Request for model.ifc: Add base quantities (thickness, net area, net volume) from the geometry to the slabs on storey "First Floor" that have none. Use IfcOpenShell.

First a look at what the model holds.

```python
import ifcopenshell
import ifcopenshell.util.element
import ifcopenshell.util.unit

model = ifcopenshell.open("model.ifc")
print(model.schema)
for unit_type in ("LENGTHUNIT", "AREAUNIT", "VOLUMEUNIT"):
    print(unit_type, ifcopenshell.util.unit.calculate_unit_scale(model, unit_type))
storey = next(s for s in model.by_type("IfcBuildingStorey") if s.Name == "First Floor")
slabs = [e for e in ifcopenshell.util.element.get_decomposition(storey) if e.is_a("IfcSlab")]
for e in sorted(slabs, key=lambda e: e.id()):
    print(e.id(), e.is_a(), e.Name, list(ifcopenshell.util.element.get_psets(e, qtos_only=True)), sep=" | ")
```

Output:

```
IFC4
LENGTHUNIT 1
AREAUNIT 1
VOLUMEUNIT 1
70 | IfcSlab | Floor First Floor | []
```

```python
import ifcopenshell
import ifcopenshell.api.pset
import ifcopenshell.geom
import ifcopenshell.util.element
import ifcopenshell.util.shape
import ifcopenshell.util.unit

model = ifcopenshell.open("model.ifc")
unit_scale = ifcopenshell.util.unit.calculate_unit_scale(model)
area_scale = ifcopenshell.util.unit.calculate_unit_scale(model, "AREAUNIT")
volume_scale = ifcopenshell.util.unit.calculate_unit_scale(model, "VOLUMEUNIT")
settings = ifcopenshell.geom.settings()

storey = next(s for s in model.by_type("IfcBuildingStorey") if s.Name == "First Floor")
slabs = [e for e in ifcopenshell.util.element.get_decomposition(storey) if e.is_a("IfcSlab")]

for e in sorted(slabs, key=lambda e: e.id()):
    if ifcopenshell.util.element.get_psets(e, qtos_only=True, should_inherit=False):
        continue
    # Geometry comes back in metres, in the element's own axes.
    shape = ifcopenshell.geom.create_shape(settings, e)
    values = {
        "Width": ifcopenshell.util.shape.get_z(shape.geometry) / unit_scale,
        "NetArea": ifcopenshell.util.shape.get_footprint_area(shape.geometry) / area_scale,
        "NetVolume": ifcopenshell.util.shape.get_volume(shape.geometry) / volume_scale,
    }
    qto = ifcopenshell.api.pset.add_qto(model, product=e, name="Qto_SlabBaseQuantities")
    ifcopenshell.api.pset.edit_qto(model, qto=qto, properties=values)
    print(e.id(), {k: round(v, 3) for k, v in values.items()})

model.write("model_rev.ifc")
```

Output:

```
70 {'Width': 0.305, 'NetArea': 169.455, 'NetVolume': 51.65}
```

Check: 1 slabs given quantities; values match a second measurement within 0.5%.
